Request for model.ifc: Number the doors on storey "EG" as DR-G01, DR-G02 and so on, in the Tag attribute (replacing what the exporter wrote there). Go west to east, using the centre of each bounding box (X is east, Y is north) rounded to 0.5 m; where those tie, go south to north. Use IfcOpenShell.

First a look at what the model holds.

```python
import ifcopenshell
import ifcopenshell.util.element
import ifcopenshell.util.placement

model = ifcopenshell.open("model.ifc")
print(model.schema)
storey = next(s for s in model.by_type("IfcBuildingStorey") if s.Name == "EG")
doors = [e for e in ifcopenshell.util.element.get_decomposition(storey) if e.is_a("IfcDoor")]
for e in sorted(doors, key=lambda e: e.id()):
    origin = ifcopenshell.util.placement.get_local_placement(e.ObjectPlacement)[:3, 3]
    print(e.id(), e.Tag, e.Name, origin.round(2) + 0.0, sep=" | ")
```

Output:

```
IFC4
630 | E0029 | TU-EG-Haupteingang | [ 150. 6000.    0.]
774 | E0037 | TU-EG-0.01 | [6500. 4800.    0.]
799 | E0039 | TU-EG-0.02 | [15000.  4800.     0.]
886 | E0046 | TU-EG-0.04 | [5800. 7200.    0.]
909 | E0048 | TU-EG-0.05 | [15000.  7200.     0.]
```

```python
import ifcopenshell
import ifcopenshell.geom
import ifcopenshell.util.element
import ifcopenshell.util.shape

model = ifcopenshell.open("model.ifc")
settings = ifcopenshell.geom.settings()
settings.set("use-world-coords", True)


def centre(element):
    shape = ifcopenshell.geom.create_shape(settings, element)
    return ifcopenshell.util.shape.get_bbox_centroid(shape.geometry)


storey = next(s for s in model.by_type("IfcBuildingStorey") if s.Name == "EG")
doors = [e for e in ifcopenshell.util.element.get_decomposition(storey) if e.is_a("IfcDoor")]

# Insertion points can sit at a corner or the storey origin, so sort by the geometry (in metres).
centres = {e: centre(e) for e in doors}
doors.sort(key=lambda e: (round(centres[e][0] / 0.5), centres[e][1]))

for i, e in enumerate(doors, start=1):
    number = f"DR-G{i:02d}"
    e.Tag = number
    print(e.id(), number)

model.write("model_v2.ifc")
```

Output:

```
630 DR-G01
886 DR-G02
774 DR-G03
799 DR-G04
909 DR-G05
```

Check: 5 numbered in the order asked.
